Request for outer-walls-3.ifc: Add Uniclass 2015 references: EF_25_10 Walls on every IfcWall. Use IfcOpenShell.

First a look at what the model holds.

```python
import ifcopenshell

model = ifcopenshell.open("outer-walls-3.ifc")
print(model.schema)
print("classifications:", [c.Name for c in model.by_type("IfcClassification")])
for ifc_class in ("IfcDoor", "IfcRoof", "IfcStair", "IfcWall", "IfcWindow"):
    print(ifc_class, len(model.by_type(ifc_class)))
```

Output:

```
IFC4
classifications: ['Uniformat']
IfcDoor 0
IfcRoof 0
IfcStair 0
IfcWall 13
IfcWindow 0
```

```python
import ifcopenshell
import ifcopenshell.api.classification

model = ifcopenshell.open("outer-walls-3.ifc")

system = ifcopenshell.api.classification.add_classification(model, classification="Uniclass 2015")

codes = {
    "IfcWall": ("EF_25_10", "Walls"),
}
for ifc_class, (code, name) in codes.items():
    products = model.by_type(ifc_class)
    ifcopenshell.api.classification.add_reference(
        model, products=products, classification=system, identification=code, name=name
    )
    print(code, len(products))

model.write("outer-walls-3_rev.ifc")
```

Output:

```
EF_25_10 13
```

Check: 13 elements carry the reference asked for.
